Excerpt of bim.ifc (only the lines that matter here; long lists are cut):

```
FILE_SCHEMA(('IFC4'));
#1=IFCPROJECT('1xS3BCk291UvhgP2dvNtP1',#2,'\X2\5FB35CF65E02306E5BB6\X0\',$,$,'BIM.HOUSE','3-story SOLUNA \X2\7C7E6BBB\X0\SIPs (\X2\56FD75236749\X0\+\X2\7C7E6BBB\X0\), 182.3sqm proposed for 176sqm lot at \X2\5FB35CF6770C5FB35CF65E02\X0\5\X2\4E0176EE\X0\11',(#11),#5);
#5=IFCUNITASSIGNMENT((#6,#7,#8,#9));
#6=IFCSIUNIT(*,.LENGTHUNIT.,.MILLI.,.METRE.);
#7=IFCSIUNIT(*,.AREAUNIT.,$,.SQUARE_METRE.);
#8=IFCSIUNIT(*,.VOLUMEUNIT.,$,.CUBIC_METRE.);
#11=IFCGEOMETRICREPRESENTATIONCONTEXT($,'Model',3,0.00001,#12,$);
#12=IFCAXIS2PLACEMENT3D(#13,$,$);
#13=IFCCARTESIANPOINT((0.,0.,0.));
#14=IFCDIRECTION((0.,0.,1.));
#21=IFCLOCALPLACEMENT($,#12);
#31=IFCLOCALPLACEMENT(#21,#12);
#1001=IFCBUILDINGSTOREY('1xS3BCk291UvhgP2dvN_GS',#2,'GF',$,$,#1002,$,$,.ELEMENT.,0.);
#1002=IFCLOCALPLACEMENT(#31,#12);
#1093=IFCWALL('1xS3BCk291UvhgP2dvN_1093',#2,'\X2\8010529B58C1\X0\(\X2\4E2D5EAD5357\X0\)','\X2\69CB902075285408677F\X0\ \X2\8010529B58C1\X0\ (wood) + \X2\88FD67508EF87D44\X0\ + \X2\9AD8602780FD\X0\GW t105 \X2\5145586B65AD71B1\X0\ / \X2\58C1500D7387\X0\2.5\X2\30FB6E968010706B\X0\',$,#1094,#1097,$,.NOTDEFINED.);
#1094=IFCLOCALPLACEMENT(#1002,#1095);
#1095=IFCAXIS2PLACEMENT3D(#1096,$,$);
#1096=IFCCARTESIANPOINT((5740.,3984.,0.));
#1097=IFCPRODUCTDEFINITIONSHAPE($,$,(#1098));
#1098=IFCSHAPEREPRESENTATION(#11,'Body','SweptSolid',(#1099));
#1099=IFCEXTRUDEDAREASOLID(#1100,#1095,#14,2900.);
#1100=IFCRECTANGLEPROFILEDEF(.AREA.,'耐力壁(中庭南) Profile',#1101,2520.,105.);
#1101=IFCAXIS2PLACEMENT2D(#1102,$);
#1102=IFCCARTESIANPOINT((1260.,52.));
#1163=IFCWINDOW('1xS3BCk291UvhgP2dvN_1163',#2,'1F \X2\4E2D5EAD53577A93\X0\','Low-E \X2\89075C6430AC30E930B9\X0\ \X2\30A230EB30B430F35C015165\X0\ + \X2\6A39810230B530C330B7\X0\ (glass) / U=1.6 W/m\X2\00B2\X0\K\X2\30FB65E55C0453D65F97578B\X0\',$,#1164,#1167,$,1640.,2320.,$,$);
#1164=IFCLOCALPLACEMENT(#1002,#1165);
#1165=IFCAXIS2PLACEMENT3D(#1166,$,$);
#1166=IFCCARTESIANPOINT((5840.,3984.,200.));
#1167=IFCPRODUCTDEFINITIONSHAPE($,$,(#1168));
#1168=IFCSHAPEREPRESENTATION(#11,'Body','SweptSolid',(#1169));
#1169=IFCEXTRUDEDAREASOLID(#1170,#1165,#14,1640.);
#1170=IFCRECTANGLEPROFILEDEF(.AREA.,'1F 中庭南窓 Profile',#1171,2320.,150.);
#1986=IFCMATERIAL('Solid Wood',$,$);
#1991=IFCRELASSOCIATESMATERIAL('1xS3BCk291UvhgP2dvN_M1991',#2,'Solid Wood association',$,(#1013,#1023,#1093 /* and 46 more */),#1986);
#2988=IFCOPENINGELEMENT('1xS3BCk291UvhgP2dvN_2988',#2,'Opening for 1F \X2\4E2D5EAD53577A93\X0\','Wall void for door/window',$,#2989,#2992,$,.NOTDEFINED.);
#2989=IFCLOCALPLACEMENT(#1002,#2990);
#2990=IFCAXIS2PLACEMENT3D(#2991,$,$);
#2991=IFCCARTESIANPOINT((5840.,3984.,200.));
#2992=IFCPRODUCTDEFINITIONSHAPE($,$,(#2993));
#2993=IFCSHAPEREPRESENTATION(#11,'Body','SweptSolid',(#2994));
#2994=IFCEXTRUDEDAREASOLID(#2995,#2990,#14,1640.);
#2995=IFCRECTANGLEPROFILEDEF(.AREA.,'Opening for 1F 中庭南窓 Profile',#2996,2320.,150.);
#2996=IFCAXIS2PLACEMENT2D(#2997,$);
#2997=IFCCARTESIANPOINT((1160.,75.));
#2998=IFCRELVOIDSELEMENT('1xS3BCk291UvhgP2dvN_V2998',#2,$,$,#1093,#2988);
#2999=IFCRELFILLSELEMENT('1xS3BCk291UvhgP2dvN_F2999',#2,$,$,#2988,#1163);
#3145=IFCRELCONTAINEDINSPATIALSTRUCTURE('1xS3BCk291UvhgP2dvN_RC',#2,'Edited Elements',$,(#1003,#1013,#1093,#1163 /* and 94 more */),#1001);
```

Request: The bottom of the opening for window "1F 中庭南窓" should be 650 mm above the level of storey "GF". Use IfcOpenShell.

```python
import numpy as np
import ifcopenshell
import ifcopenshell.api.geometry
import ifcopenshell.geom
import ifcopenshell.util.element
import ifcopenshell.util.placement
import ifcopenshell.util.shape
import ifcopenshell.util.unit

model = ifcopenshell.open("bim.ifc")
unit_scale = ifcopenshell.util.unit.calculate_unit_scale(model)

window = model.by_id(1163)
opening = window.FillsVoids[0].RelatingOpeningElement
storey = ifcopenshell.util.element.get_container(window, ifc_class="IfcBuildingStorey")
level = ifcopenshell.util.placement.get_local_placement(storey.ObjectPlacement)[2, 3]

# The opening's origin need not be at the sill, so measure its lowest point.
shape = ifcopenshell.geom.create_shape(ifcopenshell.geom.settings(), opening)
bottom = ifcopenshell.util.shape.get_shape_bottom_elevation(shape, shape.geometry) / unit_scale
dz = level + 0.65 / unit_scale - bottom

shift = np.array([0.0, 0.0, dz])
# The window is not placed relative to its opening, so move both.
for product in (opening, window):
    matrix = ifcopenshell.util.placement.get_local_placement(product.ObjectPlacement)
    matrix[:3, 3] += shift
    ifcopenshell.api.geometry.edit_object_placement(model, product=product, matrix=matrix, is_si=False)

print(f"moved by {dz * unit_scale:+.3f} m")

model.write("bim_edited.ifc")
```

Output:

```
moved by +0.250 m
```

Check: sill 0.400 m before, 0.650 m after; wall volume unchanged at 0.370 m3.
